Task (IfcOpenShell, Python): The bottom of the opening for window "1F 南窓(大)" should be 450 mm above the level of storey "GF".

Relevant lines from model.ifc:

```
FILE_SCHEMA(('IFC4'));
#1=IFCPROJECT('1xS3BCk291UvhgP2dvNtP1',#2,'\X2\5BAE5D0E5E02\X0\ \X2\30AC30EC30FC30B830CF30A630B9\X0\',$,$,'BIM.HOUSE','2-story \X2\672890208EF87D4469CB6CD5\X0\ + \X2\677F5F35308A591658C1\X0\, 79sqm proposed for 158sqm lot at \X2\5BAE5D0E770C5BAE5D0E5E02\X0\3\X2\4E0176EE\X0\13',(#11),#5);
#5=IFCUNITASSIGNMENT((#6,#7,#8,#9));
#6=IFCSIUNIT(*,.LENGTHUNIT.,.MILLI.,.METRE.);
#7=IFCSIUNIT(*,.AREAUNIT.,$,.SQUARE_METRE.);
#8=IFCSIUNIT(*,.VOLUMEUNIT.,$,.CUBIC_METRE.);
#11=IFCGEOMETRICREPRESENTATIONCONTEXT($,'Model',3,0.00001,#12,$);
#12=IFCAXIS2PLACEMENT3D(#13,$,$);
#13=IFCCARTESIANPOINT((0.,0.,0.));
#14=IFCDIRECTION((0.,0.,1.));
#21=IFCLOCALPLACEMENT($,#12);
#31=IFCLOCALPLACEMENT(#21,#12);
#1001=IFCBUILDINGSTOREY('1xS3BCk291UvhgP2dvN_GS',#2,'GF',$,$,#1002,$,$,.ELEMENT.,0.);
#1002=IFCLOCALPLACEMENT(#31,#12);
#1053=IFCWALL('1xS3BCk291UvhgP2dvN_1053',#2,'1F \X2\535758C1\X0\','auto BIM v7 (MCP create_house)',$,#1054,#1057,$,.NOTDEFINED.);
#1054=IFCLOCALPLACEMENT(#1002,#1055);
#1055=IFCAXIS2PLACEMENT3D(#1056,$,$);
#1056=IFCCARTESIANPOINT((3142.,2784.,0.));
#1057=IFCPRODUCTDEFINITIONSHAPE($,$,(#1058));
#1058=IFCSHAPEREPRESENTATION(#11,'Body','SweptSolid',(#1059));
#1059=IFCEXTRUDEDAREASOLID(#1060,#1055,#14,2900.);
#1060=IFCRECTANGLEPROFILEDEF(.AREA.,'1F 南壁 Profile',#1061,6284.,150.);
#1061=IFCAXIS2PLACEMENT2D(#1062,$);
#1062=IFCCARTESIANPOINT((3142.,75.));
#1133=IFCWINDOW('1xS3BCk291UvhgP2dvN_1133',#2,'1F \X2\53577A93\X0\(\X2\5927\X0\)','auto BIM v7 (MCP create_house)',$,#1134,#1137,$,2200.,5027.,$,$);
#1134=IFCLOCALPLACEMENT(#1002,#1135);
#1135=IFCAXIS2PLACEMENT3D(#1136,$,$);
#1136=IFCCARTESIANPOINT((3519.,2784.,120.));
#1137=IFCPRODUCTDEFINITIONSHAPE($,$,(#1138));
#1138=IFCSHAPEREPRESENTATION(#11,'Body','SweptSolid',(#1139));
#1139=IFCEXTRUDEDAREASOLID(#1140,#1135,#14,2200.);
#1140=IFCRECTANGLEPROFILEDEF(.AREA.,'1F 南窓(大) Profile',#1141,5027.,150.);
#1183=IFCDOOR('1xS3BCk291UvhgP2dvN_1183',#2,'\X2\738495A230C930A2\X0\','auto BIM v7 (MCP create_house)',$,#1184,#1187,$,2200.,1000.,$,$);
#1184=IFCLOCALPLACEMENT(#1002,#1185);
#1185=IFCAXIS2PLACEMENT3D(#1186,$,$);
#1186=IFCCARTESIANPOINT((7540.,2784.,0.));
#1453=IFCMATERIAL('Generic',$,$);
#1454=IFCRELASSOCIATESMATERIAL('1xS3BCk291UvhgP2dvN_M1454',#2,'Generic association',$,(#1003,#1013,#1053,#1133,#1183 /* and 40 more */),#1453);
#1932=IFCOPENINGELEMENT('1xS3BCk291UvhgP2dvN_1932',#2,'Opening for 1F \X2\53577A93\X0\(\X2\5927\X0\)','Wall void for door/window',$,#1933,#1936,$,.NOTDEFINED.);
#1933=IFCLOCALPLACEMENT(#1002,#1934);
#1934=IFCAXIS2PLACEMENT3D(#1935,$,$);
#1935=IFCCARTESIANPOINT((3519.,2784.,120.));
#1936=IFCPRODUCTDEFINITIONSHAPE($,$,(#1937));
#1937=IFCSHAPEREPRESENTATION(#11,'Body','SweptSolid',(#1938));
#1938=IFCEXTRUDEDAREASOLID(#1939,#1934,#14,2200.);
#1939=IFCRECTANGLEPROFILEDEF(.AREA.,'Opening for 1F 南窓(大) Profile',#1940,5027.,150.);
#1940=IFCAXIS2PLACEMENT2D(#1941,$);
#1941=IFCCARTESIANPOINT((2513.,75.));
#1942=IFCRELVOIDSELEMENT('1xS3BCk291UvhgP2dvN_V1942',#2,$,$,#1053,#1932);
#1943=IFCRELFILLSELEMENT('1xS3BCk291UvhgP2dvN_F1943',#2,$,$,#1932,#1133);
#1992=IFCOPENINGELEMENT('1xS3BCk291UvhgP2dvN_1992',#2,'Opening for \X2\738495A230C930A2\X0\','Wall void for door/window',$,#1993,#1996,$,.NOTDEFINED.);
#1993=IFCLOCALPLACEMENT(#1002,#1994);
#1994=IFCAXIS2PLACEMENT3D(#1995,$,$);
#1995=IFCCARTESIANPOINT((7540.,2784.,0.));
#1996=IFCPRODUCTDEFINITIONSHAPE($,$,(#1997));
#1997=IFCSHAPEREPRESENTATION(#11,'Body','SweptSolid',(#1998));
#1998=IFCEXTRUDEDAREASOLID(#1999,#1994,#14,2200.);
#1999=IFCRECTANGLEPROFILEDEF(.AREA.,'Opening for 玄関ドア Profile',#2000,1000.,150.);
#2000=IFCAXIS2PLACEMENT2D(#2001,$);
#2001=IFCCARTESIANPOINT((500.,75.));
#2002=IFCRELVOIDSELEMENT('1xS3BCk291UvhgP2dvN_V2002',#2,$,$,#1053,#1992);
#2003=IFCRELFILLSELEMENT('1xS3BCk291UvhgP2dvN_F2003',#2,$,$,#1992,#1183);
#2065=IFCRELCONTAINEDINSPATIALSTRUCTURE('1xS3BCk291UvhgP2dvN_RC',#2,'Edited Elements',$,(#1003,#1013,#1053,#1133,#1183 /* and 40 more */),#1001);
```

```python
import numpy as np
import ifcopenshell
import ifcopenshell.api.geometry
import ifcopenshell.geom
import ifcopenshell.util.element
import ifcopenshell.util.placement
import ifcopenshell.util.shape
import ifcopenshell.util.unit

model = ifcopenshell.open("model.ifc")
unit_scale = ifcopenshell.util.unit.calculate_unit_scale(model)

window = model.by_guid("1xS3BCk291UvhgP2dvN_1133")
opening = window.FillsVoids[0].RelatingOpeningElement
storey = ifcopenshell.util.element.get_container(window, ifc_class="IfcBuildingStorey")
level = ifcopenshell.util.placement.get_local_placement(storey.ObjectPlacement)[2, 3]

# The opening's origin need not be at the sill, so measure its lowest point.
shape = ifcopenshell.geom.create_shape(ifcopenshell.geom.settings(), opening)
bottom = ifcopenshell.util.shape.get_shape_bottom_elevation(shape, shape.geometry) / unit_scale
dz = level + 0.45 / unit_scale - bottom

shift = np.array([0.0, 0.0, dz])
# The window is not placed relative to its opening, so move both.
for product in (opening, window):
    matrix = ifcopenshell.util.placement.get_local_placement(product.ObjectPlacement)
    matrix[:3, 3] += shift
    ifcopenshell.api.geometry.edit_object_placement(model, product=product, matrix=matrix, is_si=False)

print(f"moved by {dz * unit_scale:+.3f} m")

model.write("model_updated.ifc")
```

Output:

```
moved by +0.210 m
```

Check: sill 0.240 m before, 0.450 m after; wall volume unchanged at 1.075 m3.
